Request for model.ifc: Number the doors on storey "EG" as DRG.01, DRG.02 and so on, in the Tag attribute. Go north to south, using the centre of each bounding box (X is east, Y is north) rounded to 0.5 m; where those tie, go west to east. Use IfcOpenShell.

First a look at what the model holds.

```python
import ifcopenshell
import ifcopenshell.util.element
import ifcopenshell.util.placement

model = ifcopenshell.open("model.ifc")
print(model.schema)
storey = next(s for s in model.by_type("IfcBuildingStorey") if s.Name == "EG")
doors = [e for e in ifcopenshell.util.element.get_decomposition(storey) if e.is_a("IfcDoor")]
for e in sorted(doors, key=lambda e: e.id()):
    origin = ifcopenshell.util.placement.get_local_placement(e.ObjectPlacement)[:3, 3]
    print(e.id(), e.Tag, e.Name, origin.round(2) + 0.0, sep=" | ")
```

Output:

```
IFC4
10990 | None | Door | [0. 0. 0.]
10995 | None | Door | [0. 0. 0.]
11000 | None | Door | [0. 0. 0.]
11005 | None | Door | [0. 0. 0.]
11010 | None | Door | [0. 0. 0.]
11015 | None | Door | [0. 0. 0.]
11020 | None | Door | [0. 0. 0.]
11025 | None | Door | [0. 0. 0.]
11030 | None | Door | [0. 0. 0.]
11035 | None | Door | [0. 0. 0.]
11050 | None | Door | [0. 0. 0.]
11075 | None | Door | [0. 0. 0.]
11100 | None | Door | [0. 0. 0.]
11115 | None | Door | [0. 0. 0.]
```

```python
import ifcopenshell
import ifcopenshell.geom
import ifcopenshell.util.element
import ifcopenshell.util.shape

model = ifcopenshell.open("model.ifc")
settings = ifcopenshell.geom.settings()
settings.set("use-world-coords", True)


def centre(element):
    shape = ifcopenshell.geom.create_shape(settings, element)
    return ifcopenshell.util.shape.get_bbox_centroid(shape.geometry)


storey = next(s for s in model.by_type("IfcBuildingStorey") if s.Name == "EG")
doors = [e for e in ifcopenshell.util.element.get_decomposition(storey) if e.is_a("IfcDoor")]

# Insertion points can sit at a corner or the storey origin, so sort by the geometry (in metres).
centres = {e: centre(e) for e in doors}
doors.sort(key=lambda e: (-round(centres[e][1] / 0.5), centres[e][0]))

for i, e in enumerate(doors, start=1):
    number = f"DRG.{i:02d}"
    e.Tag = number
    print(e.id(), number)

model.write("model_updated.ifc")
```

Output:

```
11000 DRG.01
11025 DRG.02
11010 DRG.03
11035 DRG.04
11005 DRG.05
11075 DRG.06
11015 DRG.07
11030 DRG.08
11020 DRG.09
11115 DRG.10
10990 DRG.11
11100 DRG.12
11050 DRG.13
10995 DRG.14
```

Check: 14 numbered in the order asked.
